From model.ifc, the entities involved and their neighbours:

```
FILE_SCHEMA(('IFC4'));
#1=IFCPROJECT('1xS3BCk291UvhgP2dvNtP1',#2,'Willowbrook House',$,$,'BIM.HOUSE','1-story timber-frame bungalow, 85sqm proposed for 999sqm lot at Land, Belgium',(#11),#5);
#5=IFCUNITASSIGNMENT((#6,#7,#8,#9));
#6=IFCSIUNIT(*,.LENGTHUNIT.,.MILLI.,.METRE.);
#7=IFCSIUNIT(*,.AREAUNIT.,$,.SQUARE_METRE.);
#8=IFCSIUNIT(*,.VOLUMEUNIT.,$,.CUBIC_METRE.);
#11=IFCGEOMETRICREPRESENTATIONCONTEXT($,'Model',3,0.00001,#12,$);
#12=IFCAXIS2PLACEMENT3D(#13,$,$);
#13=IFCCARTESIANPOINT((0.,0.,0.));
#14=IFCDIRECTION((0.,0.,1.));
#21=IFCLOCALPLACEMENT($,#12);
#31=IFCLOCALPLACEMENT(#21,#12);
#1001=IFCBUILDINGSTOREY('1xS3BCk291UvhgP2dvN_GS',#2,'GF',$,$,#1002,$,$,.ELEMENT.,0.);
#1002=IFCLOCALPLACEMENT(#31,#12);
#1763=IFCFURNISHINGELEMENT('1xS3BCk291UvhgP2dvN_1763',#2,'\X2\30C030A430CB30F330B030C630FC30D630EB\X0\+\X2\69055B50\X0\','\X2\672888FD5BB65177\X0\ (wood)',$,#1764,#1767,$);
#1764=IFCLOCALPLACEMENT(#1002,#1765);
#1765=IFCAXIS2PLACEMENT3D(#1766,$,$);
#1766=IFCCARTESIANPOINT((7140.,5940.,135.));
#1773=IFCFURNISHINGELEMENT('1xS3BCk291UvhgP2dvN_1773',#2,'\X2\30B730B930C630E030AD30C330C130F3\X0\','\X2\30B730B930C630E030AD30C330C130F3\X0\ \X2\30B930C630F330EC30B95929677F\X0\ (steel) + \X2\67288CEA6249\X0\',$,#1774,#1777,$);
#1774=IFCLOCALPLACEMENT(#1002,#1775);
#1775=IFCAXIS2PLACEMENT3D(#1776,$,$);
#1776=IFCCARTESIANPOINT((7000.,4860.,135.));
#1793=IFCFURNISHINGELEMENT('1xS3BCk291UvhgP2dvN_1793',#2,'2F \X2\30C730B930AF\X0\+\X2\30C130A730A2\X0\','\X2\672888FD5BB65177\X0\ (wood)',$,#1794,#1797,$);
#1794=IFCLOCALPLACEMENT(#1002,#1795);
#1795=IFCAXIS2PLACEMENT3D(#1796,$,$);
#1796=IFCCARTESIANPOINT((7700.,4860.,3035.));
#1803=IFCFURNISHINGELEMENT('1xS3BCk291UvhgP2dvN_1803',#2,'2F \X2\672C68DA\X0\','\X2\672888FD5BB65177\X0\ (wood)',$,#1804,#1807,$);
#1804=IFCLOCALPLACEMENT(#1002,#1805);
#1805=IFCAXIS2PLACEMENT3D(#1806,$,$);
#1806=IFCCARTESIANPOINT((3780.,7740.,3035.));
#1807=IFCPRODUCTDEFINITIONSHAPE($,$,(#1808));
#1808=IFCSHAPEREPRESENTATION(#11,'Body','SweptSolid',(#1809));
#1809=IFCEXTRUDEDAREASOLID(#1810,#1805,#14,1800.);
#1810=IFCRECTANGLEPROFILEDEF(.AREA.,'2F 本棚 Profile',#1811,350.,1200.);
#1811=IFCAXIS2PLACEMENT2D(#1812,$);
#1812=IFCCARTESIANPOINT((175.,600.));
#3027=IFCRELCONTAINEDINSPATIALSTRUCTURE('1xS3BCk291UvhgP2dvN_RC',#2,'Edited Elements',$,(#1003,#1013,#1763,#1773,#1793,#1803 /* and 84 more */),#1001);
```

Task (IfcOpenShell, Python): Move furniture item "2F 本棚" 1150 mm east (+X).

```python
import ifcopenshell
import ifcopenshell.api.geometry
import ifcopenshell.util.placement
import ifcopenshell.util.unit

model = ifcopenshell.open("model.ifc")
unit_scale = ifcopenshell.util.unit.calculate_unit_scale(model)

item = model.by_id(1803)
matrix = ifcopenshell.util.placement.get_local_placement(item.ObjectPlacement)
matrix[0, 3] += 1.15 / unit_scale
ifcopenshell.api.geometry.edit_object_placement(model, product=item, matrix=matrix, is_si=False)

print(ifcopenshell.util.placement.get_local_placement(item.ObjectPlacement).round(3) + 0.0)

model.write("model_updated.ifc")
```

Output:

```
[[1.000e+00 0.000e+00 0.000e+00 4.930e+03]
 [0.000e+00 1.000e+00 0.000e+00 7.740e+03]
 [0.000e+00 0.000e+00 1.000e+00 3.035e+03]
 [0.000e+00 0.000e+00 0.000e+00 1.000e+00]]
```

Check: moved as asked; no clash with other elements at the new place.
